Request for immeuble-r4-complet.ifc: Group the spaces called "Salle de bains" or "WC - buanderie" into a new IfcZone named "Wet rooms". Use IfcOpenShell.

First a look at what the model holds.

```python
import ifcopenshell

model = ifcopenshell.open("immeuble-r4-complet.ifc")
print(model.schema)
seen = {}
for space in model.by_type("IfcSpace"):
    seen[space.Name] = seen.get(space.Name, 0) + 1
for name, count in sorted(seen.items(), key=str):
    print(count, "x", name)
print("zones:", [z.Name for z in model.by_type("IfcZone")][:20])
```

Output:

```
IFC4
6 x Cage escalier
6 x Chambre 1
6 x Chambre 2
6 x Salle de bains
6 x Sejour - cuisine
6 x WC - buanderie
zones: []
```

```python
import ifcopenshell
import ifcopenshell.api.group
import ifcopenshell.api.root

model = ifcopenshell.open("immeuble-r4-complet.ifc")

names = {"Salle de bains", "WC - buanderie"}
spaces = [s for s in model.by_type("IfcSpace") if s.Name in names]

zone = ifcopenshell.api.root.create_entity(model, ifc_class="IfcZone", name="Wet rooms")
ifcopenshell.api.group.assign_group(model, products=spaces, group=zone)
print(len(spaces), "spaces in", zone.Name)

model.write("immeuble-r4-complet-out.ifc")
```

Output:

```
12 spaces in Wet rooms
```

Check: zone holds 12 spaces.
